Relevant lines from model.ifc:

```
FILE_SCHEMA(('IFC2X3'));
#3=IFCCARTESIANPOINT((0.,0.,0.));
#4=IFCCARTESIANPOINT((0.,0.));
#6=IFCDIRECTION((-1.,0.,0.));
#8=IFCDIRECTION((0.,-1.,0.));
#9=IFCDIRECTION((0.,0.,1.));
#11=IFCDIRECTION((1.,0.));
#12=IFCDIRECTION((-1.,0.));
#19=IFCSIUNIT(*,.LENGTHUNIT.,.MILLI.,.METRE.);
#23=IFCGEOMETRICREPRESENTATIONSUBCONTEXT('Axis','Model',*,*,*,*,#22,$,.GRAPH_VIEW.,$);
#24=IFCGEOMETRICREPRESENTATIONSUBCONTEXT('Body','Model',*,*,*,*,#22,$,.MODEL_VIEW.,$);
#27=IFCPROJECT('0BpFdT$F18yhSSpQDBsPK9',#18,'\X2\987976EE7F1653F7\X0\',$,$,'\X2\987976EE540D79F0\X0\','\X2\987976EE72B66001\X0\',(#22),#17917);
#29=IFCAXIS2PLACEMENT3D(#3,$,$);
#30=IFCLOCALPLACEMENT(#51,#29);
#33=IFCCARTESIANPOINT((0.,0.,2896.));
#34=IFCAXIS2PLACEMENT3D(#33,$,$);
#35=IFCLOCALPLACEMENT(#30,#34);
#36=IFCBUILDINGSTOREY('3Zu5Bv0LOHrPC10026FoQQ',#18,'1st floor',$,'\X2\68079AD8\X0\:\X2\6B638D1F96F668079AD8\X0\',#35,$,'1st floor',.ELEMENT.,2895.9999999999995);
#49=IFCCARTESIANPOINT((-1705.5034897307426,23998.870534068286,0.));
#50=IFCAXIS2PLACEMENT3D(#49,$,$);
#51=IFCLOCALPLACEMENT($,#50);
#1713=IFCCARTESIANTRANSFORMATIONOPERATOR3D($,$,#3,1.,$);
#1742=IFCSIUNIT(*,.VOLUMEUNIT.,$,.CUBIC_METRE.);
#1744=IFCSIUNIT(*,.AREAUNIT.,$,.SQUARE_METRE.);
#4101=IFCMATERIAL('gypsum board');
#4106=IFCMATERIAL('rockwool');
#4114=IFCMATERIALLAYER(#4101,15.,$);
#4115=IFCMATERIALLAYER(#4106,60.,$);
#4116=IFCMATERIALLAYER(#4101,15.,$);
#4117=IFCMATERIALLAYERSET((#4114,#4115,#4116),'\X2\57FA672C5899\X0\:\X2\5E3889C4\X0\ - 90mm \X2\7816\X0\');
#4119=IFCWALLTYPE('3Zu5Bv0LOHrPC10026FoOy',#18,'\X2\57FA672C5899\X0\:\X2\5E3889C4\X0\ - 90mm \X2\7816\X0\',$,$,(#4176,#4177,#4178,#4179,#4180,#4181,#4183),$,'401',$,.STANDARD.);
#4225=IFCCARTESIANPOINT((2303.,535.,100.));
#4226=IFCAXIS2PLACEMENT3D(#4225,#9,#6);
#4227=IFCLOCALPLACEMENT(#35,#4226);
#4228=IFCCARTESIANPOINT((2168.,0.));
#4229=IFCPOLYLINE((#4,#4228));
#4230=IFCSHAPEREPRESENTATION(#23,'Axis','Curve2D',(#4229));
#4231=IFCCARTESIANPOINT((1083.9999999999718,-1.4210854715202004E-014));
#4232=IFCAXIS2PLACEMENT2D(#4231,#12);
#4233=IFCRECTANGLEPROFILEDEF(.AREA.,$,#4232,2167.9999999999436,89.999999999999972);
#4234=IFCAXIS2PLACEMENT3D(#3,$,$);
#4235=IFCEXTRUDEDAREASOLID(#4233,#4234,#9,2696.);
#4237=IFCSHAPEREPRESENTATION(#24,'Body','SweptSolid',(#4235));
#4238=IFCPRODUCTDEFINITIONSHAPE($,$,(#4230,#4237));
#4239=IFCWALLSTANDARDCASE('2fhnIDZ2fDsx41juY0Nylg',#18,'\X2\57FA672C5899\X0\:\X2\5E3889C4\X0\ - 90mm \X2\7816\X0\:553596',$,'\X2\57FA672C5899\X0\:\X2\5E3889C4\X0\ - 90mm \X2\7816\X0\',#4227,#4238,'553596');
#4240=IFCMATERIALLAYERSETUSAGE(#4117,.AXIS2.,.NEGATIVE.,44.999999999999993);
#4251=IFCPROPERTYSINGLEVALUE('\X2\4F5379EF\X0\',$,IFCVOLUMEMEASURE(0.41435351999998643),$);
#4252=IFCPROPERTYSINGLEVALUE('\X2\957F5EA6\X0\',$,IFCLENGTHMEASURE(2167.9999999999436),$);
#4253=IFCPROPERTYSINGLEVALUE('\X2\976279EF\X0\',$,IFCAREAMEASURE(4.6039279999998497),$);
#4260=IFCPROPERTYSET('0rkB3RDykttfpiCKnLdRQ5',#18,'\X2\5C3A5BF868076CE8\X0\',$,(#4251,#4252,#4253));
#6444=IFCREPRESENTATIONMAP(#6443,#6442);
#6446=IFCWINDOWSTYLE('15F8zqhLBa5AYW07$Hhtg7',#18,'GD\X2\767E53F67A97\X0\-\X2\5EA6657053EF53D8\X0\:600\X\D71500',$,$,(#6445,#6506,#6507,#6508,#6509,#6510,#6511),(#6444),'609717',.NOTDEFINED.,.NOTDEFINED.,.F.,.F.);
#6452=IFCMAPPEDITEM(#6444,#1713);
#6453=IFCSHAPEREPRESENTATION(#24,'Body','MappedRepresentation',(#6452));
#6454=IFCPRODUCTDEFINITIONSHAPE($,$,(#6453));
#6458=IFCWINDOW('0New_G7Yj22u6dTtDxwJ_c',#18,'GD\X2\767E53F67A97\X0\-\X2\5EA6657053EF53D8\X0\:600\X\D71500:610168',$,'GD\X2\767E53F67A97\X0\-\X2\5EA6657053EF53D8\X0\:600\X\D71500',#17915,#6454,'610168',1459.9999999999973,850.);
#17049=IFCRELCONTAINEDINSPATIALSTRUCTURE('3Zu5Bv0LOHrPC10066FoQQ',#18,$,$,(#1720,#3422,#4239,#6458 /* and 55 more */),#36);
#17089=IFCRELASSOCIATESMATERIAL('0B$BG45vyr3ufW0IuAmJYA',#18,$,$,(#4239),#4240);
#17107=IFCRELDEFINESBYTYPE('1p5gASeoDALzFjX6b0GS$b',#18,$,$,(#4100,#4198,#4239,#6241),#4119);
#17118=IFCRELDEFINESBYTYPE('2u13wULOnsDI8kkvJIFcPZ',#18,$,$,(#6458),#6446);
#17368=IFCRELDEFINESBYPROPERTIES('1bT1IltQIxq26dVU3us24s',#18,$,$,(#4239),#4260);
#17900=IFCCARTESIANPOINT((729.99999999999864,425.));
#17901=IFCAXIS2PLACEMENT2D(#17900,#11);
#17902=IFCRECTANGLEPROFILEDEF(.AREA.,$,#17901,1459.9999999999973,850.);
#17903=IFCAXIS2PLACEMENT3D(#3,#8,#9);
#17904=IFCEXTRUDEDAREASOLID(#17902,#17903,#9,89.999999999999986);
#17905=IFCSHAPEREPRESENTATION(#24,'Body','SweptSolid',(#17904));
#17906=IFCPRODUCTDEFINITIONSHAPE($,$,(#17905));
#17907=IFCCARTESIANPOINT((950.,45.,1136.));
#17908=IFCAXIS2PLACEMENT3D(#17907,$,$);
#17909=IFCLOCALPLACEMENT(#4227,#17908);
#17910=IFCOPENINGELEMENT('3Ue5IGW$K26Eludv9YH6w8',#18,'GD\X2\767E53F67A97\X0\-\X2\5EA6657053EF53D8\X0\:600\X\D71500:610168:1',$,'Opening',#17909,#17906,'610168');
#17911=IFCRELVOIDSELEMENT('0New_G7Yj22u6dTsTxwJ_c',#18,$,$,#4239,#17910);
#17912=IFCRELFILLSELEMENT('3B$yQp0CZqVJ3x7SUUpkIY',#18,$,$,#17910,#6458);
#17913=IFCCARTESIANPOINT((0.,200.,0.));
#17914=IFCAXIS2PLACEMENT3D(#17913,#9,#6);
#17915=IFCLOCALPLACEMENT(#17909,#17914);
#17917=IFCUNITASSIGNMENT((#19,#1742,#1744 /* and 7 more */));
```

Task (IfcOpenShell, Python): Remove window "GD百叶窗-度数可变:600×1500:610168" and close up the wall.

```python
import ifcopenshell
import ifcopenshell.api.feature
import ifcopenshell.api.pset
import ifcopenshell.api.root
import ifcopenshell.geom
import ifcopenshell.util.element
import ifcopenshell.util.shape
import ifcopenshell.util.unit

model = ifcopenshell.open("model.ifc")
area_scale = ifcopenshell.util.unit.calculate_unit_scale(model, "AREAUNIT")
volume_scale = ifcopenshell.util.unit.calculate_unit_scale(model, "VOLUMEUNIT")
settings = ifcopenshell.geom.settings()


def volume(element):
    """Net volume in cubic metres, openings subtracted."""
    shape = ifcopenshell.geom.create_shape(settings, element)
    return ifcopenshell.util.shape.get_volume(shape.geometry)


window = model.by_id(6458)
opening = window.FillsVoids[0].RelatingOpeningElement
wall = opening.VoidsElements[0].RelatingBuildingElement
before = volume(wall)

ifcopenshell.api.root.remove_product(model, product=window)
ifcopenshell.api.feature.remove_feature(model, feature=opening)

after = volume(wall)
thickness = 0.09  # wall thickness in metres

# Update the wall's stored quantities.
pset = model.by_id(ifcopenshell.util.element.get_pset(wall, "尺寸标注", should_inherit=False)["id"])
ifcopenshell.api.pset.edit_pset(model, pset=pset, properties={
    "体积": model.create_entity("IfcVolumeMeasure", after / volume_scale),
    "面积": model.create_entity("IfcAreaMeasure", after / thickness / area_scale),
})

print(f"wall volume {before:.3f} -> {after:.3f} m3")

model.write("model_updated.ifc")
```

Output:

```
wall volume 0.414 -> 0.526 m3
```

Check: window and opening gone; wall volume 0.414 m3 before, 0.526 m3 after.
